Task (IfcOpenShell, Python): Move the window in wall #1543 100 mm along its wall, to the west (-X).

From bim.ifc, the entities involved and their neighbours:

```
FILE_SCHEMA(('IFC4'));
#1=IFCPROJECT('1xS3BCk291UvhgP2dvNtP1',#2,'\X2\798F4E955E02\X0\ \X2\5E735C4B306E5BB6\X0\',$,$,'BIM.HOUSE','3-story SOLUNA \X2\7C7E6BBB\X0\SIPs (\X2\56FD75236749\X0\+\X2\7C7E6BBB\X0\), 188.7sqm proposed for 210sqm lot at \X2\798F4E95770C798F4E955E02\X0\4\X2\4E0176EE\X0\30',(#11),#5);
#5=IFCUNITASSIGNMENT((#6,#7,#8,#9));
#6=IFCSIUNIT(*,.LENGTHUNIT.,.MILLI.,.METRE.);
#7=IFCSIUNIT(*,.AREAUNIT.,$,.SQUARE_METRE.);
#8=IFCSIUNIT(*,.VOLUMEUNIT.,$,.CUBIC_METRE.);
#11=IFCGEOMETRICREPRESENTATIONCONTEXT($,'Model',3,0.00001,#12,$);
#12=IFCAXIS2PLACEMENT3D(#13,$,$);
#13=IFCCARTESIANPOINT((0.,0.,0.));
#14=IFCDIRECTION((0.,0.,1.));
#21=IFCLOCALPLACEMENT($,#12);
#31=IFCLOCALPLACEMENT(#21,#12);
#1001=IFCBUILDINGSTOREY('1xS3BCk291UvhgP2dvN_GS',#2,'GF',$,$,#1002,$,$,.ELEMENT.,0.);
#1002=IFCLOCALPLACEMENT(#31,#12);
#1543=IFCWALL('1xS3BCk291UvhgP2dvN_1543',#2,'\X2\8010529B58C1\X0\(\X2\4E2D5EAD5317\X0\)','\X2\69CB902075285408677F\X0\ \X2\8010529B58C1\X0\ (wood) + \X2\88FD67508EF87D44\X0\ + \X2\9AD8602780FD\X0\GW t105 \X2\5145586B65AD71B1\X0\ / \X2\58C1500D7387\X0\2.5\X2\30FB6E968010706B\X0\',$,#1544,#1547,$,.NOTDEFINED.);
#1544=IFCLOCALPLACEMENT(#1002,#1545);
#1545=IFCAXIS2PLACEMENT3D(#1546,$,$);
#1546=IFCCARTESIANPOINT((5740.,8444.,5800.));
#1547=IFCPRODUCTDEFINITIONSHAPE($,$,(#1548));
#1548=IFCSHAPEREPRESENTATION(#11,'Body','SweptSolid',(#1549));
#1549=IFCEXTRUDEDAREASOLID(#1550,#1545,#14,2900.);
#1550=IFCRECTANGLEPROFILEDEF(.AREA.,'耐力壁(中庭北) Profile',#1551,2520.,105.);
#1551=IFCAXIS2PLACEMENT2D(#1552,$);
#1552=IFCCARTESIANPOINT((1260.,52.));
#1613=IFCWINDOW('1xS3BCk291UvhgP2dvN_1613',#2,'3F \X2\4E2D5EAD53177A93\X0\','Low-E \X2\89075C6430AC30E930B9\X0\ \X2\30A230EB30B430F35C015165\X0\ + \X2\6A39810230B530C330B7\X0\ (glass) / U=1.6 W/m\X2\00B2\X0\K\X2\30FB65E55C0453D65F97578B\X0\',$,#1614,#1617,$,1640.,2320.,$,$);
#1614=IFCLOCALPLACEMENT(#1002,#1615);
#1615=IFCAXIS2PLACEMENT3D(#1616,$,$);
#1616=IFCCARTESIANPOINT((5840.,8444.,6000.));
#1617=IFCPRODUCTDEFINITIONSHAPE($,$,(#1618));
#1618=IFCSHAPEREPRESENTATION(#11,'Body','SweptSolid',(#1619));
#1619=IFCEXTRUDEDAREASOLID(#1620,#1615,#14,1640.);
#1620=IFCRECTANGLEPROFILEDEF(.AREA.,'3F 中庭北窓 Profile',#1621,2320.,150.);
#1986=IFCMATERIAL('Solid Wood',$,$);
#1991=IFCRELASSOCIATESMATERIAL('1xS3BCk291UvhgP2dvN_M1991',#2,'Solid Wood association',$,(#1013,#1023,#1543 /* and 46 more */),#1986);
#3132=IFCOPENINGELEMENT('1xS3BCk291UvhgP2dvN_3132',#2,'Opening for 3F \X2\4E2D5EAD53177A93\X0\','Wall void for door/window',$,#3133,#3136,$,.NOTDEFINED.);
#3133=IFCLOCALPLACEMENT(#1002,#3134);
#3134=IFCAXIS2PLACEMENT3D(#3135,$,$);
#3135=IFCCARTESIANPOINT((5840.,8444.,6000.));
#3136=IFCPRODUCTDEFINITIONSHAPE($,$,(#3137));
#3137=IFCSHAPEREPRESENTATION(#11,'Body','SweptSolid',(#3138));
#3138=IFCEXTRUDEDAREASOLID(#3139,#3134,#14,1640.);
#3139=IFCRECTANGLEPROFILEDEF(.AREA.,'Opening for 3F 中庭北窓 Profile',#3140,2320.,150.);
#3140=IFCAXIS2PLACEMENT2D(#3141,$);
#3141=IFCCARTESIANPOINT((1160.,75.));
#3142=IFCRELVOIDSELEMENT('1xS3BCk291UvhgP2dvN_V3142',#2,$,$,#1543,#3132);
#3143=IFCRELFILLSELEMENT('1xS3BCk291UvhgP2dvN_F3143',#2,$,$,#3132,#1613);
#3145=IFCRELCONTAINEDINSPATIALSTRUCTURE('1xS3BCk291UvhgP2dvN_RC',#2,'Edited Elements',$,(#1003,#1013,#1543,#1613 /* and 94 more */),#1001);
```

```python
import ifcopenshell
import ifcopenshell.api.geometry
import ifcopenshell.util.placement
import ifcopenshell.util.unit

model = ifcopenshell.open("bim.ifc")
unit_scale = ifcopenshell.util.unit.calculate_unit_scale(model)

window = model.by_guid("1xS3BCk291UvhgP2dvN_1613")
opening = window.FillsVoids[0].RelatingOpeningElement
wall = opening.VoidsElements[0].RelatingBuildingElement

wall_matrix = ifcopenshell.util.placement.get_local_placement(wall.ObjectPlacement)
shift = wall_matrix[:3, 0] * -0.1 / unit_scale
before = ifcopenshell.util.placement.get_local_placement(window.ObjectPlacement)[:3, 3].copy()

# The window is not placed relative to its opening, so move both.
for product in (opening, window):
    matrix = ifcopenshell.util.placement.get_local_placement(product.ObjectPlacement)
    matrix[:3, 3] += shift
    ifcopenshell.api.geometry.edit_object_placement(model, product=product, matrix=matrix, is_si=False)

after = ifcopenshell.util.placement.get_local_placement(window.ObjectPlacement)[:3, 3]
print("window moved by", (after - before).round(3) + 0.0)

model.write("bim_rev.ifc")
```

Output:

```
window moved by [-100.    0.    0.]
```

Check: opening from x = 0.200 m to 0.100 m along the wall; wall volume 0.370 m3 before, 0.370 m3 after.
